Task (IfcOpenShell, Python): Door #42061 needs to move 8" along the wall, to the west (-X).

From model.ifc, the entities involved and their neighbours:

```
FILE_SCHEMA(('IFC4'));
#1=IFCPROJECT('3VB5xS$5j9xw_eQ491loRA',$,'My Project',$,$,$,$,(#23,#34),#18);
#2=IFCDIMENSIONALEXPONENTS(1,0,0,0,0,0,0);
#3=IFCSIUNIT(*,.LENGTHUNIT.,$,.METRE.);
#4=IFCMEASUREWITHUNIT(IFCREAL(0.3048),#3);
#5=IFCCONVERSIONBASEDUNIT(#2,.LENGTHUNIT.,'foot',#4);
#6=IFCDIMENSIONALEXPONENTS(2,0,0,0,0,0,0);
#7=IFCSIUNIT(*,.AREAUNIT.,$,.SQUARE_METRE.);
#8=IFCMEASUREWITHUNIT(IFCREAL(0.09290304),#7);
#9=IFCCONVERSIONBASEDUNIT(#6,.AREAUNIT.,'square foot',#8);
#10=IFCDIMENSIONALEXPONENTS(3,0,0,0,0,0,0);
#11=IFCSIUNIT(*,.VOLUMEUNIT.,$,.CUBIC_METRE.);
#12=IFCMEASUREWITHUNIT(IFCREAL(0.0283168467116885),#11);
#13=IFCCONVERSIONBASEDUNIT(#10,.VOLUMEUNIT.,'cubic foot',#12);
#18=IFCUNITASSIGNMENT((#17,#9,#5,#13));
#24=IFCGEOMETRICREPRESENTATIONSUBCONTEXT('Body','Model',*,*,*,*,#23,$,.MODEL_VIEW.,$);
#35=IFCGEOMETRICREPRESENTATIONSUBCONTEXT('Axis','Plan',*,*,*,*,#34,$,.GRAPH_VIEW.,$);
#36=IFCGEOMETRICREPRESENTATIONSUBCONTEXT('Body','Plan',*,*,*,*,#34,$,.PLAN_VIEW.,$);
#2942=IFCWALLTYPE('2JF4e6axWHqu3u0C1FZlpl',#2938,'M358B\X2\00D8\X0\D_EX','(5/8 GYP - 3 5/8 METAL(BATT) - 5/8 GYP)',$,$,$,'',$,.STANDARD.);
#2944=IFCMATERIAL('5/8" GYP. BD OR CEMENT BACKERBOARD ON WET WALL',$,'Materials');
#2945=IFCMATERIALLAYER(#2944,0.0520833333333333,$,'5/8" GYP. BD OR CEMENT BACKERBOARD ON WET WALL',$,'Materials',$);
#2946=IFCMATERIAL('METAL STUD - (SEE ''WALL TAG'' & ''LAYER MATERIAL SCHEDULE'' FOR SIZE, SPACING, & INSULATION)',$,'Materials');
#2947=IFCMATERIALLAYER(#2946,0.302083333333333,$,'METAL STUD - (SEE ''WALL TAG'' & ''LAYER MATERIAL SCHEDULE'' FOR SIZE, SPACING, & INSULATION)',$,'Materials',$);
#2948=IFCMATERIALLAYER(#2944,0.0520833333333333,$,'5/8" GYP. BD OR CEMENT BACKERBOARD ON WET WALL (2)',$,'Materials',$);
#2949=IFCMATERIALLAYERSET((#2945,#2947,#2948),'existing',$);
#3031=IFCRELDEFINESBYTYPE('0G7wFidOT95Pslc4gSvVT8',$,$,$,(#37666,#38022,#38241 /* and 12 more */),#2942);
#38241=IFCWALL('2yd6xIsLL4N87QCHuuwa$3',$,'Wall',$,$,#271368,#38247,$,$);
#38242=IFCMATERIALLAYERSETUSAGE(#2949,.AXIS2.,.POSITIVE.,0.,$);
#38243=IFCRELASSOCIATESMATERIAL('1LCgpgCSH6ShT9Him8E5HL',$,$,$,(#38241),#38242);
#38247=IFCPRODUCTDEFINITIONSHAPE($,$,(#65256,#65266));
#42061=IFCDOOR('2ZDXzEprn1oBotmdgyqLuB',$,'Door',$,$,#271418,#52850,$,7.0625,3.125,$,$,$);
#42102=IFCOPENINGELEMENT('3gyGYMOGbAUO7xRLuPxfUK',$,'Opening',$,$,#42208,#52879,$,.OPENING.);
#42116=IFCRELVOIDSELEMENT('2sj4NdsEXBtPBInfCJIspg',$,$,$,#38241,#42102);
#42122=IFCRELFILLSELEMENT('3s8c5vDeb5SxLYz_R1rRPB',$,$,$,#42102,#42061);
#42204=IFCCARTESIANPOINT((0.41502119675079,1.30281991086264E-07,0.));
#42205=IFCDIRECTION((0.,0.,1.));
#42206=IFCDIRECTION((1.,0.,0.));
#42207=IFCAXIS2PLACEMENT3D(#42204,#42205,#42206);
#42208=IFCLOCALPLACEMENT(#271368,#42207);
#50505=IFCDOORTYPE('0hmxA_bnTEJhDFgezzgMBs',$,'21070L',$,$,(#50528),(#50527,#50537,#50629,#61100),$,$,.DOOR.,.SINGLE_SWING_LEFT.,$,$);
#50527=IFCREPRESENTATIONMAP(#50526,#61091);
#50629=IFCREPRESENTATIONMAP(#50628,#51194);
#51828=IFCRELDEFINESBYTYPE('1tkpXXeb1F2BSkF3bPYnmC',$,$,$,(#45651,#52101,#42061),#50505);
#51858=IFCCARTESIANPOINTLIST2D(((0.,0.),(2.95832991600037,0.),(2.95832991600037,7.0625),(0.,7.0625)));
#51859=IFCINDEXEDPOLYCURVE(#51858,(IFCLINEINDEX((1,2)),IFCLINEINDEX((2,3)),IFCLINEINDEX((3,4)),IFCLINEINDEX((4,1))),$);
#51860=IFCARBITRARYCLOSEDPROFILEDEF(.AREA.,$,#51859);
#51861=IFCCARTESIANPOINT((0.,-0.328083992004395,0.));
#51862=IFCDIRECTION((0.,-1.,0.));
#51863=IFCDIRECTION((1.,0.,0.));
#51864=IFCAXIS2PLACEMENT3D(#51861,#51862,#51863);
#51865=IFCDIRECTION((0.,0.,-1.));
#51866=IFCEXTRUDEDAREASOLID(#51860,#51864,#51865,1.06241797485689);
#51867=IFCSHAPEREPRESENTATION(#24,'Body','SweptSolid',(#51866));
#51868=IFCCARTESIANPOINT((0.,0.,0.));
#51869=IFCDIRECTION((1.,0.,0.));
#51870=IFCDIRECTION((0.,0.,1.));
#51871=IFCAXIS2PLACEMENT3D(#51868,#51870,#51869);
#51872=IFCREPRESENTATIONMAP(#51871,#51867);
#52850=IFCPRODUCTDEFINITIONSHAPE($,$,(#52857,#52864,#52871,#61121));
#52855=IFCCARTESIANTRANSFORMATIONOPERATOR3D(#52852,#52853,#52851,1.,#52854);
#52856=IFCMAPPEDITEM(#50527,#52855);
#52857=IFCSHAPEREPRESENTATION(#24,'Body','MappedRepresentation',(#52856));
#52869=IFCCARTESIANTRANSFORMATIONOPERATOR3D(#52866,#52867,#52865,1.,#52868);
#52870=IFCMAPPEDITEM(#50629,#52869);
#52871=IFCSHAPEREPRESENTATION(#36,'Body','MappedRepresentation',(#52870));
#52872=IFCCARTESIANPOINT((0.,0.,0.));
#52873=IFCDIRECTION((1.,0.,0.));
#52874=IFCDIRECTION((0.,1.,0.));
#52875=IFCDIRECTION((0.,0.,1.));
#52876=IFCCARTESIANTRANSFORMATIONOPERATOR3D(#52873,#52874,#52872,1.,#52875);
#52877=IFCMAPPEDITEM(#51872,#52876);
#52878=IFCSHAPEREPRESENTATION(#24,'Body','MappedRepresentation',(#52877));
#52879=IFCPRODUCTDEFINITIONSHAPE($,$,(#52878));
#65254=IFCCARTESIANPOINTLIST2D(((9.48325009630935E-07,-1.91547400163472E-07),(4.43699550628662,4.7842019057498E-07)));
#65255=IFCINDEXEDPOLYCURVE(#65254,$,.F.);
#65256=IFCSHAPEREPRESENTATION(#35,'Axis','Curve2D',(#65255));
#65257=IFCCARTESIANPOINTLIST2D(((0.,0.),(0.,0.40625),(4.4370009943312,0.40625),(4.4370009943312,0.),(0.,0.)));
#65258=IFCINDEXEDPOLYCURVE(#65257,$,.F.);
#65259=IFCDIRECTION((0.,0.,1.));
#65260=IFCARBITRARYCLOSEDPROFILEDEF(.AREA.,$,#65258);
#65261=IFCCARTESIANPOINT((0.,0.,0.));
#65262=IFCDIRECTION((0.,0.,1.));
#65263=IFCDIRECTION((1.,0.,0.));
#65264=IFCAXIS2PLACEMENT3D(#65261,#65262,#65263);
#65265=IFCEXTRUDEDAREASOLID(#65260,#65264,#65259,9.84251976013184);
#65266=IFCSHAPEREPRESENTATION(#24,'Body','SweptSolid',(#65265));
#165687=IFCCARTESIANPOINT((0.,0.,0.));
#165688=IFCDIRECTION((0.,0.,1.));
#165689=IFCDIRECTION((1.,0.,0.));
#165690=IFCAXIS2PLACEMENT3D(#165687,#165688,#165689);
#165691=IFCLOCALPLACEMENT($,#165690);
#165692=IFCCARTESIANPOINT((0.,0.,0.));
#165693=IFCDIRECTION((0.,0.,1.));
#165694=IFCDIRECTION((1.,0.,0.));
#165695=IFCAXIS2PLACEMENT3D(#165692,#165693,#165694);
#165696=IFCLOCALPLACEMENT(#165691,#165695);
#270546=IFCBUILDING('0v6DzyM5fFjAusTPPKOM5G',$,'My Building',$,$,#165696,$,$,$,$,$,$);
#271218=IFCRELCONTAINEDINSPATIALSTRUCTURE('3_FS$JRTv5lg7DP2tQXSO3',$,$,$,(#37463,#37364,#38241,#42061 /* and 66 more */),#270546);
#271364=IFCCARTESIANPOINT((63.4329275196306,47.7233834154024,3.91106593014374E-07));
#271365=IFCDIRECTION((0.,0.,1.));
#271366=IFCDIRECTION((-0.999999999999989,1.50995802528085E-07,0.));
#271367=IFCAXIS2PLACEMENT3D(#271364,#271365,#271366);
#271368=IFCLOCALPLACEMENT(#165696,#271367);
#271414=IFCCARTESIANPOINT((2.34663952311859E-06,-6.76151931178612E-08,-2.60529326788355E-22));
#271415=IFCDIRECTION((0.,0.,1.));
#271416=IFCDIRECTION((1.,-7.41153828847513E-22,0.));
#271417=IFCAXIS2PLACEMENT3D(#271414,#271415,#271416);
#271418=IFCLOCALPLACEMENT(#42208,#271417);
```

```python
import ifcopenshell
import ifcopenshell.api.geometry
import ifcopenshell.util.placement
import ifcopenshell.util.unit

model = ifcopenshell.open("model.ifc")
unit_scale = ifcopenshell.util.unit.calculate_unit_scale(model)

door = model.by_guid("2ZDXzEprn1oBotmdgyqLuB")
opening = door.FillsVoids[0].RelatingOpeningElement
wall = opening.VoidsElements[0].RelatingBuildingElement

wall_matrix = ifcopenshell.util.placement.get_local_placement(wall.ObjectPlacement)
shift = wall_matrix[:3, 0] * 8 * 0.0254 / unit_scale
before = ifcopenshell.util.placement.get_local_placement(door.ObjectPlacement)[:3, 3].copy()

# The door is placed relative to its opening, so it follows when the opening moves.
matrix = ifcopenshell.util.placement.get_local_placement(opening.ObjectPlacement)
matrix[:3, 3] += shift
ifcopenshell.api.geometry.edit_object_placement(
    model, product=opening, matrix=matrix, is_si=False, should_transform_children=True
)

after = ifcopenshell.util.placement.get_local_placement(door.ObjectPlacement)[:3, 3]
print("door moved by", (after - before).round(3) + 0.0)

model.write("model_updated.ifc")
```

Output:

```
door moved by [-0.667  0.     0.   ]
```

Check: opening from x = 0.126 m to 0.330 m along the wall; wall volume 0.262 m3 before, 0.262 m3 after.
